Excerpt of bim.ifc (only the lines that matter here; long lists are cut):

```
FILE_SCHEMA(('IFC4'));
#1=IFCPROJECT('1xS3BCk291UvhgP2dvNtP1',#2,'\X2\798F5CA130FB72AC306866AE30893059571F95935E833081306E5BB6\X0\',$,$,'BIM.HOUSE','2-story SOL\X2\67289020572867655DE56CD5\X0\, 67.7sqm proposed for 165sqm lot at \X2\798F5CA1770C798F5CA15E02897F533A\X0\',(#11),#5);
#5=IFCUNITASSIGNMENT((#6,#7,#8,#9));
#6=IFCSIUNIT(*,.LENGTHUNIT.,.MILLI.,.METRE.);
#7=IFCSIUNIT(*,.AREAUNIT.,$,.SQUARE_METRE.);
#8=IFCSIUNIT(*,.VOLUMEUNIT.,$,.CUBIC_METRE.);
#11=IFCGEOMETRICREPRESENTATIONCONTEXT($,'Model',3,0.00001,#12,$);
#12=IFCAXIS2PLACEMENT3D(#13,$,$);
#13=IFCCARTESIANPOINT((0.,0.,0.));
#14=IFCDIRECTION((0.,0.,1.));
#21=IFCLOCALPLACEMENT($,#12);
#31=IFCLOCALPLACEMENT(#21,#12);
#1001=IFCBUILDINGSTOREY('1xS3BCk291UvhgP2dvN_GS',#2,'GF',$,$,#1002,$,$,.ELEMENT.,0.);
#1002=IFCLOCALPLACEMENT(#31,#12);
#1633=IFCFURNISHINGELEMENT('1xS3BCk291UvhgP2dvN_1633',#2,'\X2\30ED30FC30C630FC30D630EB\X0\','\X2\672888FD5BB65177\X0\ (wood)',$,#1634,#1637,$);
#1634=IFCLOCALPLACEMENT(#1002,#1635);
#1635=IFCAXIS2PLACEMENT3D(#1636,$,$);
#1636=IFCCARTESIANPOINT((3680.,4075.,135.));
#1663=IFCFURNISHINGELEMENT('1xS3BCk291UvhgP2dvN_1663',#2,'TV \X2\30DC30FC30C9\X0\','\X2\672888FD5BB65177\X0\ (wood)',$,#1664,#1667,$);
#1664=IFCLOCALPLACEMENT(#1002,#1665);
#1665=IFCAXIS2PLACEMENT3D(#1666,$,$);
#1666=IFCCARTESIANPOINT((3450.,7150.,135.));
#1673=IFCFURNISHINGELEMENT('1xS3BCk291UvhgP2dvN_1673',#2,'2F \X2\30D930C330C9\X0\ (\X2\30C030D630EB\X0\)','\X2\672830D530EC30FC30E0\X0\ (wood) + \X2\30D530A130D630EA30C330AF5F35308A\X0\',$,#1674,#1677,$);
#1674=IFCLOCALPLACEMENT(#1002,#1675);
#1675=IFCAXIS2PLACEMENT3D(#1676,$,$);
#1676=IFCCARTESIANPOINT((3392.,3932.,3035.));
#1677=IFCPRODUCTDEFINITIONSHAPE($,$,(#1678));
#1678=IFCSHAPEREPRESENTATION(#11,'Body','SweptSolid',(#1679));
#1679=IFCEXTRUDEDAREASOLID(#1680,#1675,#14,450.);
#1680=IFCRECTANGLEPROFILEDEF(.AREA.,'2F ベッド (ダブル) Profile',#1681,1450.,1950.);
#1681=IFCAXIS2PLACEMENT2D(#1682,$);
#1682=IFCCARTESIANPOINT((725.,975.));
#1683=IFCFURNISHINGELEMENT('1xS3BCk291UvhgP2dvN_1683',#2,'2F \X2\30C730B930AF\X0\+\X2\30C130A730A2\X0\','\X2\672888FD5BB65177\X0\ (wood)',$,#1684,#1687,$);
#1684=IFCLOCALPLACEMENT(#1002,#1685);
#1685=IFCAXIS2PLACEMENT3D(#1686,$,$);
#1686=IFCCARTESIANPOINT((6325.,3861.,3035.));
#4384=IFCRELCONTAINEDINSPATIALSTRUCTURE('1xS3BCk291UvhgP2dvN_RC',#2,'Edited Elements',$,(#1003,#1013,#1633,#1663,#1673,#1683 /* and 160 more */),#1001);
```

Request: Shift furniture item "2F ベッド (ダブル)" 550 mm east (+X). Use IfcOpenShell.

```python
import ifcopenshell
import ifcopenshell.api.geometry
import ifcopenshell.util.placement

model = ifcopenshell.open("bim.ifc")

item = model.by_id(1673)
matrix = ifcopenshell.util.placement.get_local_placement(item.ObjectPlacement)
matrix[0, 3] += 550.0
ifcopenshell.api.geometry.edit_object_placement(model, product=item, matrix=matrix, is_si=False)

print(ifcopenshell.util.placement.get_local_placement(item.ObjectPlacement).round(3) + 0.0)

model.write("bim_rev.ifc")
```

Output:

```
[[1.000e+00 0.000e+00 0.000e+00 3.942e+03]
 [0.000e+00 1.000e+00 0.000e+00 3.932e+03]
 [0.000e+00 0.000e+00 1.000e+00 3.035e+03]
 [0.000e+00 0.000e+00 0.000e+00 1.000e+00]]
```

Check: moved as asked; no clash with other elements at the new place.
